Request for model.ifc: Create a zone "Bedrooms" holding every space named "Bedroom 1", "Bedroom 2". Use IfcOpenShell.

First a look at what the model holds.

```python
import ifcopenshell

model = ifcopenshell.open("model.ifc")
print(model.schema)
seen = {}
for space in model.by_type("IfcSpace"):
    seen[space.LongName] = seen.get(space.LongName, 0) + 1
for name, count in sorted(seen.items(), key=str):
    print(count, "x", name)
print("zones:", [z.Name for z in model.by_type("IfcZone")][:20])
```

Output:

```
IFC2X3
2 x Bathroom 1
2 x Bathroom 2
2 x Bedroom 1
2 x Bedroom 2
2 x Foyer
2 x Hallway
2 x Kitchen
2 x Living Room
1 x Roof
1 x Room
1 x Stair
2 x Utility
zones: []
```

```python
import ifcopenshell
import ifcopenshell.api.group
import ifcopenshell.api.root

model = ifcopenshell.open("model.ifc")

names = {"Bedroom 1", "Bedroom 2"}
spaces = [s for s in model.by_type("IfcSpace") if s.LongName in names]

zone = ifcopenshell.api.root.create_entity(model, ifc_class="IfcZone", name="Bedrooms")
ifcopenshell.api.group.assign_group(model, products=spaces, group=zone)
print(len(spaces), "spaces in", zone.Name)

model.write("model_updated.ifc")
```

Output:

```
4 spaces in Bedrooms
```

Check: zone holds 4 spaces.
